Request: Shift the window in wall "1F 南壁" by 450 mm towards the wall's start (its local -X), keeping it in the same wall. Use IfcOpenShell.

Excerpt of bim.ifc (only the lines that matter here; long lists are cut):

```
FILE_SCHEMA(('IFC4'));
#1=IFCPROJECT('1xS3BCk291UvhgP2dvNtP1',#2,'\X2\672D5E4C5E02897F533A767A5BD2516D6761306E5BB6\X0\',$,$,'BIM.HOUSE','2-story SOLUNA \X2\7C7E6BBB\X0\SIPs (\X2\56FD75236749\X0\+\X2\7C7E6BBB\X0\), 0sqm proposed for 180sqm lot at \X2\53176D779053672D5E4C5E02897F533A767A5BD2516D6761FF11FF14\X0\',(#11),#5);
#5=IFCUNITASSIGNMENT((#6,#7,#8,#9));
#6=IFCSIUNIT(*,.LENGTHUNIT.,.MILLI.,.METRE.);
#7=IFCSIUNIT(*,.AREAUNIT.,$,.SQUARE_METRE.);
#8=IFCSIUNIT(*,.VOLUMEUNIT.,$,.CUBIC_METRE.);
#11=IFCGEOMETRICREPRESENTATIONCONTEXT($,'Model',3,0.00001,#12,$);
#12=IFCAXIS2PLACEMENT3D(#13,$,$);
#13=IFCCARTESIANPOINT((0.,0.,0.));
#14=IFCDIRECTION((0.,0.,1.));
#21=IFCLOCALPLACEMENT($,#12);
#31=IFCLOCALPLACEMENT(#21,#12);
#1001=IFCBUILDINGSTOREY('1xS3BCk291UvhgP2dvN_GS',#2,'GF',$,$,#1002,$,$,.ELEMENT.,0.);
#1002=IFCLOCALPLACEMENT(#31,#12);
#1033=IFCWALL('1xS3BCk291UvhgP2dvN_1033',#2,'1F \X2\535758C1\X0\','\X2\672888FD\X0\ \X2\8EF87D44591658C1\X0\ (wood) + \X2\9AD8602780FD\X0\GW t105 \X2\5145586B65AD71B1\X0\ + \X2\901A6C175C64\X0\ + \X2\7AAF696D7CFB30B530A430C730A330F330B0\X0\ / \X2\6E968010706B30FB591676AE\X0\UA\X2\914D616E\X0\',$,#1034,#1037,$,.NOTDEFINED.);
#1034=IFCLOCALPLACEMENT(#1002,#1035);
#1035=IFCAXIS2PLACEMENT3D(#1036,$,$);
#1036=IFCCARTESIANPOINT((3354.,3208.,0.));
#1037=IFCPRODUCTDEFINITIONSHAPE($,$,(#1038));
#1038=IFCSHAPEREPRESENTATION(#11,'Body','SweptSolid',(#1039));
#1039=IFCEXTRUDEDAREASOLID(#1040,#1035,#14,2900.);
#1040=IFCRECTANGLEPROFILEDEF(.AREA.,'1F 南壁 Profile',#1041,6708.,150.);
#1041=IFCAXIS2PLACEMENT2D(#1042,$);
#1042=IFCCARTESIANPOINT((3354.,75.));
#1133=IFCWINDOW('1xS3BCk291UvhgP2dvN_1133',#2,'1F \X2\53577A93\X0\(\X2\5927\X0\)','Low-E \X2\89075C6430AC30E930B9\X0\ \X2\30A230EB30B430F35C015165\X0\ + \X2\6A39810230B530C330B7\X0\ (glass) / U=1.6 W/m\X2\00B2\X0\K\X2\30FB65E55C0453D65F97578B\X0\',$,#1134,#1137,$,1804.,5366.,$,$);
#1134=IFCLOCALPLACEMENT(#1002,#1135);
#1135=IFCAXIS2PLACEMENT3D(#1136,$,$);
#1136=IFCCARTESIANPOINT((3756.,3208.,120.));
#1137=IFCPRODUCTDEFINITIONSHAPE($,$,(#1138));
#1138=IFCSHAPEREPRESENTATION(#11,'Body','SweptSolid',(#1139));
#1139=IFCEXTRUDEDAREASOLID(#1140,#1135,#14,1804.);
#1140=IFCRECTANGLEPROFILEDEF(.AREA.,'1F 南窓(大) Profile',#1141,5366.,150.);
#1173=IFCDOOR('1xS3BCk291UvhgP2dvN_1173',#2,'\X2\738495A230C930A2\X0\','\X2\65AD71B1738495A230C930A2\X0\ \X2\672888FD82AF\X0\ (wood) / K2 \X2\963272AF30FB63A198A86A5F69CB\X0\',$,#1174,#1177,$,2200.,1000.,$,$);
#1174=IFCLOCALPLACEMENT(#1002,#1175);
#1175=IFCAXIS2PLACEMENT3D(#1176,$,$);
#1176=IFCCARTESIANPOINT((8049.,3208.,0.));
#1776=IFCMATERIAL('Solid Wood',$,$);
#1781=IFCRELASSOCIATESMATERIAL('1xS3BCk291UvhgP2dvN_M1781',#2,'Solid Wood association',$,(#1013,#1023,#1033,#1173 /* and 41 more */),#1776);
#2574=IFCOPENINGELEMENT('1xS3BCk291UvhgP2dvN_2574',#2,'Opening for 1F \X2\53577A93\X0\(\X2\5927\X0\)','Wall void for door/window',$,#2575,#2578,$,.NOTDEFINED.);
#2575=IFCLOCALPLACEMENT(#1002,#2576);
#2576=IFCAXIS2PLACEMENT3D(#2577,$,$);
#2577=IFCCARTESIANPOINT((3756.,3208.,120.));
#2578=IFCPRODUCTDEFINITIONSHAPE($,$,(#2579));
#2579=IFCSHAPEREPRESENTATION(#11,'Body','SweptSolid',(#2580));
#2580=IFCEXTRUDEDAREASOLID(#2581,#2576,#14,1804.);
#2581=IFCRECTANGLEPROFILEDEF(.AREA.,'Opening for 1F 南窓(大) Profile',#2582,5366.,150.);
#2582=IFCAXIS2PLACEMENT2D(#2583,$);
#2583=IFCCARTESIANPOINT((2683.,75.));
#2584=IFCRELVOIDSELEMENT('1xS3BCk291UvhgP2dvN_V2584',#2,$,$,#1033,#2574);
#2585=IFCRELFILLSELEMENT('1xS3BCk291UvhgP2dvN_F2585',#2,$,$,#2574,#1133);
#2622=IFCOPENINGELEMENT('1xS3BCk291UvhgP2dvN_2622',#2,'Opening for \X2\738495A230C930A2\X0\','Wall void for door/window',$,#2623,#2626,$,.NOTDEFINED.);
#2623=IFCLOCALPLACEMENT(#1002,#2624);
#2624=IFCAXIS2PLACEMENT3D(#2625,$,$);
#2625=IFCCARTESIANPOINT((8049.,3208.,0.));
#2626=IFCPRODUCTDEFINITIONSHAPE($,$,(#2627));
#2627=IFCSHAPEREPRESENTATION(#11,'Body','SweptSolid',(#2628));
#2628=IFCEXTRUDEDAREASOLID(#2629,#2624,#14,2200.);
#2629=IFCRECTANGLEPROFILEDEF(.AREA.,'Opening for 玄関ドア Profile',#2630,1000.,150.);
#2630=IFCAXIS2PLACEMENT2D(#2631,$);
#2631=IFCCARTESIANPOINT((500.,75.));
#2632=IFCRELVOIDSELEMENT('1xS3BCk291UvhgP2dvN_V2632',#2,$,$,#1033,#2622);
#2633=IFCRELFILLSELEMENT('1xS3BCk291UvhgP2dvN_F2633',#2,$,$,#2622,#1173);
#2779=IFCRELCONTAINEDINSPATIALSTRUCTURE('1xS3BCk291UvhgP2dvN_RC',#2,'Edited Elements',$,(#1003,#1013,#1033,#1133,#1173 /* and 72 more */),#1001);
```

```python
import ifcopenshell
import ifcopenshell.api.geometry
import ifcopenshell.util.placement

model = ifcopenshell.open("bim.ifc")

window = model.by_guid("1xS3BCk291UvhgP2dvN_1133")
opening = window.FillsVoids[0].RelatingOpeningElement
wall = opening.VoidsElements[0].RelatingBuildingElement

wall_matrix = ifcopenshell.util.placement.get_local_placement(wall.ObjectPlacement)
shift = wall_matrix[:3, 0] * -450.0
before = ifcopenshell.util.placement.get_local_placement(window.ObjectPlacement)[:3, 3].copy()

# The window is not placed relative to its opening, so move both.
for product in (opening, window):
    matrix = ifcopenshell.util.placement.get_local_placement(product.ObjectPlacement)
    matrix[:3, 3] += shift
    ifcopenshell.api.geometry.edit_object_placement(model, product=product, matrix=matrix, is_si=False)

after = ifcopenshell.util.placement.get_local_placement(window.ObjectPlacement)[:3, 3]
print("window moved by", (after - before).round(3) + 0.0)

model.write("bim_edited.ifc")
```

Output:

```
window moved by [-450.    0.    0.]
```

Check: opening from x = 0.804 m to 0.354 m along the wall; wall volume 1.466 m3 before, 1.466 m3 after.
